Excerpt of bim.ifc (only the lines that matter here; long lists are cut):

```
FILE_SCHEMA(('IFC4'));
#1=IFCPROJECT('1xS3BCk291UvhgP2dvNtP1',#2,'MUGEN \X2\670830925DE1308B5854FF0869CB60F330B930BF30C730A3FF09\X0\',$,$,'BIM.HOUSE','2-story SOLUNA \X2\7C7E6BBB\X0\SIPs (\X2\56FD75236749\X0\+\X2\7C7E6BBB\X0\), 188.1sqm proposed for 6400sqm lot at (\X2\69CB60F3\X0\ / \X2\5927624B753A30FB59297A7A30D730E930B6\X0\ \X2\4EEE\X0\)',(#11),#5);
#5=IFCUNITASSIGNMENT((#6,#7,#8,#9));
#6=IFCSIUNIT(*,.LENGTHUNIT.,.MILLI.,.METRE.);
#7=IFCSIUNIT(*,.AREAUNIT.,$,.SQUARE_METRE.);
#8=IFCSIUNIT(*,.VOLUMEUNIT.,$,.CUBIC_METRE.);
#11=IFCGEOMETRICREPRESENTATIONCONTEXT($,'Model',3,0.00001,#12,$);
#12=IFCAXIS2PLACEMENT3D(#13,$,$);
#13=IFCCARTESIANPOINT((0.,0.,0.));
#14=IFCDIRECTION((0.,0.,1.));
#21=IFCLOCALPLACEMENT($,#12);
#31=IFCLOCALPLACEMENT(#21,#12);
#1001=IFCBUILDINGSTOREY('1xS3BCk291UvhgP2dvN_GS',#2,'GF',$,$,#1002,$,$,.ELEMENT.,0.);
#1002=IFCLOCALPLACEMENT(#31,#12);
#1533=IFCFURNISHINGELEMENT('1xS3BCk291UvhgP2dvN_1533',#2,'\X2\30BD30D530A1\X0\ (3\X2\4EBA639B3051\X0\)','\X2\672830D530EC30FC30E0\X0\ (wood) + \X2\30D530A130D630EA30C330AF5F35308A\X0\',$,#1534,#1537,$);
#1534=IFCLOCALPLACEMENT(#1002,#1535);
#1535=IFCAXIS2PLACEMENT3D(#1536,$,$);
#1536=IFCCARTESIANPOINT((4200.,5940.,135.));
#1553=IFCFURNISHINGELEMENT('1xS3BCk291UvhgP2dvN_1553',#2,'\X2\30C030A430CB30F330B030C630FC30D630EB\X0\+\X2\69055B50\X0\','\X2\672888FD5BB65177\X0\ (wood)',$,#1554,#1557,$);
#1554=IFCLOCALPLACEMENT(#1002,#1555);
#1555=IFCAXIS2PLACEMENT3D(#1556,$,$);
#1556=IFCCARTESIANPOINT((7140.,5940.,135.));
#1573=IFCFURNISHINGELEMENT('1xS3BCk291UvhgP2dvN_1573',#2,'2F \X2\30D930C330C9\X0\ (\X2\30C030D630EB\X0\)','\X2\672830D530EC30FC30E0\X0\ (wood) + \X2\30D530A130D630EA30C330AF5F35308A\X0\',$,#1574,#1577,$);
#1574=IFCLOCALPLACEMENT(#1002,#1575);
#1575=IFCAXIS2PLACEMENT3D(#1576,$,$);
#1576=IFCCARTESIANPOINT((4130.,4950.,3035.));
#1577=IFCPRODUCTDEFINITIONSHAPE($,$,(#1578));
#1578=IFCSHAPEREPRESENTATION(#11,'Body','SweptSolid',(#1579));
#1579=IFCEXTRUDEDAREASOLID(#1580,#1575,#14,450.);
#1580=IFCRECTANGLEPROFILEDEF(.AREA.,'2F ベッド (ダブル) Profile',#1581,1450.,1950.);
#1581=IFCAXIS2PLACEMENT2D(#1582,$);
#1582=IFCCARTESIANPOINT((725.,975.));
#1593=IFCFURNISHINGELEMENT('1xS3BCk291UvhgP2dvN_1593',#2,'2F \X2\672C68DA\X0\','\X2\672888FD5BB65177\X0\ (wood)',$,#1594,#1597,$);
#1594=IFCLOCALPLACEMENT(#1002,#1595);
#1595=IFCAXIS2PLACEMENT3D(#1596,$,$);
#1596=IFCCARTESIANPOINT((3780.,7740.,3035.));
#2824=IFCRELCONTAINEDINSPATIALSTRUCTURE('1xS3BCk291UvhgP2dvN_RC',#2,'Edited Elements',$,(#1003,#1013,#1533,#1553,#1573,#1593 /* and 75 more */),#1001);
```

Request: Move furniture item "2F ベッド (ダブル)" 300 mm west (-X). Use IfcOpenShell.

```python
import ifcopenshell
import ifcopenshell.api.geometry
import ifcopenshell.util.placement

model = ifcopenshell.open("bim.ifc")

item = model.by_guid("1xS3BCk291UvhgP2dvN_1573")
matrix = ifcopenshell.util.placement.get_local_placement(item.ObjectPlacement)
matrix[0, 3] -= 300.0
ifcopenshell.api.geometry.edit_object_placement(model, product=item, matrix=matrix, is_si=False)

print(ifcopenshell.util.placement.get_local_placement(item.ObjectPlacement).round(3) + 0.0)

model.write("bim_rev.ifc")
```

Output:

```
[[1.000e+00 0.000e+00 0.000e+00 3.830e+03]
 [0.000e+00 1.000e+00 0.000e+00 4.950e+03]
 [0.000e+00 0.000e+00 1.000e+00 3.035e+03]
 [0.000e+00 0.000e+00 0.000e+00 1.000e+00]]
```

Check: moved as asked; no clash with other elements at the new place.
